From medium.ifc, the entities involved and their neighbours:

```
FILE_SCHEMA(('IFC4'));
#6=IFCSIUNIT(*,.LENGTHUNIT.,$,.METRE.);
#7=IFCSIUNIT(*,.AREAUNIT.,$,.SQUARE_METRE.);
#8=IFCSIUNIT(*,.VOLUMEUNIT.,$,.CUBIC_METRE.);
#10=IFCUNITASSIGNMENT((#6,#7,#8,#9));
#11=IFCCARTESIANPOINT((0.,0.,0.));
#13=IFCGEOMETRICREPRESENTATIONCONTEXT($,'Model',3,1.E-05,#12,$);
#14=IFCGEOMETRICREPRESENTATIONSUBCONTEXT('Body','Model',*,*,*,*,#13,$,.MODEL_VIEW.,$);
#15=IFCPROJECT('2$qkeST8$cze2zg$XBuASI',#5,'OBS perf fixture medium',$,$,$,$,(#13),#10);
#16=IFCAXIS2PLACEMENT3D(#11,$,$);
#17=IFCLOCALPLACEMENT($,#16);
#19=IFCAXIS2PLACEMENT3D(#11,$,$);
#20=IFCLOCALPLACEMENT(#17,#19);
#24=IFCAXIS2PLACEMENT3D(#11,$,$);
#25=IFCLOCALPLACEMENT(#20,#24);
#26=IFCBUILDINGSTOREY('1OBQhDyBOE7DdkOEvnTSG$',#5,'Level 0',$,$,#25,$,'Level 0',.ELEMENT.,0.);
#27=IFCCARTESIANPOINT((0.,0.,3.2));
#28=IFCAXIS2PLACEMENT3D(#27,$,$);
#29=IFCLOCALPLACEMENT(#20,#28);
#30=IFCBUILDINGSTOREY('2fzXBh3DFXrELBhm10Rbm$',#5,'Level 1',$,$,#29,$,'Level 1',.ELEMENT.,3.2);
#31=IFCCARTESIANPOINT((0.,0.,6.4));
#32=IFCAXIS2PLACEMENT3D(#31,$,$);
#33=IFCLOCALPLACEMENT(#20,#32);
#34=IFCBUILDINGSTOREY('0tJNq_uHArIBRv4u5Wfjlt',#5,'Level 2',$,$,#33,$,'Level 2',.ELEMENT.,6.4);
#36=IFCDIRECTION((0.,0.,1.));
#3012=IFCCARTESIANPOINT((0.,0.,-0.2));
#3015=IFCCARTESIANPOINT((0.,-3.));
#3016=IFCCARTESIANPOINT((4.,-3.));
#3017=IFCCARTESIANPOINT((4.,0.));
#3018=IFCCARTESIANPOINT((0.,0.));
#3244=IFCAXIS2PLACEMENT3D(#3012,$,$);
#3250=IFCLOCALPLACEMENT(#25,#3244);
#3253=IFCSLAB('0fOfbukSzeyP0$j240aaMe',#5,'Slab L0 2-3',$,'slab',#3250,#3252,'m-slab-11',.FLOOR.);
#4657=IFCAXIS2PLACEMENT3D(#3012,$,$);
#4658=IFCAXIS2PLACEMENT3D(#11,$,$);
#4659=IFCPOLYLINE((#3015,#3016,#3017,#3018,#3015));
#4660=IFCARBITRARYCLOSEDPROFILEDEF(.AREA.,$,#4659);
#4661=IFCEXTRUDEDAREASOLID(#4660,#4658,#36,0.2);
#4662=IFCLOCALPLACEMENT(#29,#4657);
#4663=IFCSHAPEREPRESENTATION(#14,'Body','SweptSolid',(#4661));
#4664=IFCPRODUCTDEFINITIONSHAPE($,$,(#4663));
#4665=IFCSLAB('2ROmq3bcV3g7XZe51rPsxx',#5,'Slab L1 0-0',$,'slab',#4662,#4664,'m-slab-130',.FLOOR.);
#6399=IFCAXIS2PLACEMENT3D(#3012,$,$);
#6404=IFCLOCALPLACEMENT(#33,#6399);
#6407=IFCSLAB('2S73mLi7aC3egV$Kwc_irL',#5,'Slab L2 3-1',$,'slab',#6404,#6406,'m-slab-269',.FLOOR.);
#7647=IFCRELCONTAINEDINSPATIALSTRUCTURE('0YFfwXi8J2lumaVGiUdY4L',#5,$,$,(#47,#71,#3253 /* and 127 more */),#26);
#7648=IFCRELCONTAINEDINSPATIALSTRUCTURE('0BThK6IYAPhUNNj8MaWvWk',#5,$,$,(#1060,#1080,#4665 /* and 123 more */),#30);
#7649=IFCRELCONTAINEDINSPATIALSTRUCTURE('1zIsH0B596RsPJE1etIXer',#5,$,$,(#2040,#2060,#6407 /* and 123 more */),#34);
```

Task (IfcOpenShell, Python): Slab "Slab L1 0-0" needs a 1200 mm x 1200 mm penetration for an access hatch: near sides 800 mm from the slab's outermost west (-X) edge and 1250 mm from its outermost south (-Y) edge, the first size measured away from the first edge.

```python
import numpy as np
import ifcopenshell
import ifcopenshell.api.feature
import ifcopenshell.api.geometry
import ifcopenshell.api.root
import ifcopenshell.geom
import ifcopenshell.util.placement
import ifcopenshell.util.representation
import ifcopenshell.util.shape
import ifcopenshell.util.unit

model = ifcopenshell.open("medium.ifc")
unit_scale = ifcopenshell.util.unit.calculate_unit_scale(model)
settings = ifcopenshell.geom.settings()


def volume(element):
    """Net volume in cubic metres, openings subtracted."""
    shape = ifcopenshell.geom.create_shape(settings, element)
    return ifcopenshell.util.shape.get_volume(shape.geometry)


slab = model.by_guid("2ROmq3bcV3g7XZe51rPsxx")
before = volume(slab)

# Extent in the slab's own axes, in metres. The edges named are its -X and -Y sides.
slab_shape = ifcopenshell.geom.create_shape(settings, slab)
vertices = ifcopenshell.util.shape.get_vertices(slab_shape.geometry)
x_min, y_min, bottom = vertices.min(axis=0)
top = vertices[:, 2].max()

opening = ifcopenshell.api.root.create_entity(model, ifc_class="IfcOpeningElement", name="Access hatch opening", predefined_type="OPENING")
context = ifcopenshell.util.representation.get_context(model, "Model", "Body", "MODEL_VIEW")
width, depth = 1.2, 1.2
outline = [(0.0, 0.0), (width, 0.0), (width, depth), (0.0, depth), (0.0, 0.0)]
# Overshoot both faces by 50 mm so the cut is clean.
shape = ifcopenshell.api.geometry.add_slab_representation(
    model, context=context, depth=top - bottom + 0.1, polyline=outline
)
ifcopenshell.api.geometry.assign_representation(model, product=opening, representation=shape)

matrix = ifcopenshell.util.placement.get_local_placement(slab.ObjectPlacement)
matrix[:, 3] = matrix @ np.append(np.array([x_min + 0.8, y_min + 1.25, bottom - 0.05]) / unit_scale, 1.0)
ifcopenshell.api.geometry.edit_object_placement(model, product=opening, matrix=matrix, is_si=False)
ifcopenshell.api.feature.add_feature(model, feature=opening, element=slab)

after = volume(slab)

print(f"slab volume {before:.3f} -> {after:.3f} m3")

model.write("medium-out.ifc")
```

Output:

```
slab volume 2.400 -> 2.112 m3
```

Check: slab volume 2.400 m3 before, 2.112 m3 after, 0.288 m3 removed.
